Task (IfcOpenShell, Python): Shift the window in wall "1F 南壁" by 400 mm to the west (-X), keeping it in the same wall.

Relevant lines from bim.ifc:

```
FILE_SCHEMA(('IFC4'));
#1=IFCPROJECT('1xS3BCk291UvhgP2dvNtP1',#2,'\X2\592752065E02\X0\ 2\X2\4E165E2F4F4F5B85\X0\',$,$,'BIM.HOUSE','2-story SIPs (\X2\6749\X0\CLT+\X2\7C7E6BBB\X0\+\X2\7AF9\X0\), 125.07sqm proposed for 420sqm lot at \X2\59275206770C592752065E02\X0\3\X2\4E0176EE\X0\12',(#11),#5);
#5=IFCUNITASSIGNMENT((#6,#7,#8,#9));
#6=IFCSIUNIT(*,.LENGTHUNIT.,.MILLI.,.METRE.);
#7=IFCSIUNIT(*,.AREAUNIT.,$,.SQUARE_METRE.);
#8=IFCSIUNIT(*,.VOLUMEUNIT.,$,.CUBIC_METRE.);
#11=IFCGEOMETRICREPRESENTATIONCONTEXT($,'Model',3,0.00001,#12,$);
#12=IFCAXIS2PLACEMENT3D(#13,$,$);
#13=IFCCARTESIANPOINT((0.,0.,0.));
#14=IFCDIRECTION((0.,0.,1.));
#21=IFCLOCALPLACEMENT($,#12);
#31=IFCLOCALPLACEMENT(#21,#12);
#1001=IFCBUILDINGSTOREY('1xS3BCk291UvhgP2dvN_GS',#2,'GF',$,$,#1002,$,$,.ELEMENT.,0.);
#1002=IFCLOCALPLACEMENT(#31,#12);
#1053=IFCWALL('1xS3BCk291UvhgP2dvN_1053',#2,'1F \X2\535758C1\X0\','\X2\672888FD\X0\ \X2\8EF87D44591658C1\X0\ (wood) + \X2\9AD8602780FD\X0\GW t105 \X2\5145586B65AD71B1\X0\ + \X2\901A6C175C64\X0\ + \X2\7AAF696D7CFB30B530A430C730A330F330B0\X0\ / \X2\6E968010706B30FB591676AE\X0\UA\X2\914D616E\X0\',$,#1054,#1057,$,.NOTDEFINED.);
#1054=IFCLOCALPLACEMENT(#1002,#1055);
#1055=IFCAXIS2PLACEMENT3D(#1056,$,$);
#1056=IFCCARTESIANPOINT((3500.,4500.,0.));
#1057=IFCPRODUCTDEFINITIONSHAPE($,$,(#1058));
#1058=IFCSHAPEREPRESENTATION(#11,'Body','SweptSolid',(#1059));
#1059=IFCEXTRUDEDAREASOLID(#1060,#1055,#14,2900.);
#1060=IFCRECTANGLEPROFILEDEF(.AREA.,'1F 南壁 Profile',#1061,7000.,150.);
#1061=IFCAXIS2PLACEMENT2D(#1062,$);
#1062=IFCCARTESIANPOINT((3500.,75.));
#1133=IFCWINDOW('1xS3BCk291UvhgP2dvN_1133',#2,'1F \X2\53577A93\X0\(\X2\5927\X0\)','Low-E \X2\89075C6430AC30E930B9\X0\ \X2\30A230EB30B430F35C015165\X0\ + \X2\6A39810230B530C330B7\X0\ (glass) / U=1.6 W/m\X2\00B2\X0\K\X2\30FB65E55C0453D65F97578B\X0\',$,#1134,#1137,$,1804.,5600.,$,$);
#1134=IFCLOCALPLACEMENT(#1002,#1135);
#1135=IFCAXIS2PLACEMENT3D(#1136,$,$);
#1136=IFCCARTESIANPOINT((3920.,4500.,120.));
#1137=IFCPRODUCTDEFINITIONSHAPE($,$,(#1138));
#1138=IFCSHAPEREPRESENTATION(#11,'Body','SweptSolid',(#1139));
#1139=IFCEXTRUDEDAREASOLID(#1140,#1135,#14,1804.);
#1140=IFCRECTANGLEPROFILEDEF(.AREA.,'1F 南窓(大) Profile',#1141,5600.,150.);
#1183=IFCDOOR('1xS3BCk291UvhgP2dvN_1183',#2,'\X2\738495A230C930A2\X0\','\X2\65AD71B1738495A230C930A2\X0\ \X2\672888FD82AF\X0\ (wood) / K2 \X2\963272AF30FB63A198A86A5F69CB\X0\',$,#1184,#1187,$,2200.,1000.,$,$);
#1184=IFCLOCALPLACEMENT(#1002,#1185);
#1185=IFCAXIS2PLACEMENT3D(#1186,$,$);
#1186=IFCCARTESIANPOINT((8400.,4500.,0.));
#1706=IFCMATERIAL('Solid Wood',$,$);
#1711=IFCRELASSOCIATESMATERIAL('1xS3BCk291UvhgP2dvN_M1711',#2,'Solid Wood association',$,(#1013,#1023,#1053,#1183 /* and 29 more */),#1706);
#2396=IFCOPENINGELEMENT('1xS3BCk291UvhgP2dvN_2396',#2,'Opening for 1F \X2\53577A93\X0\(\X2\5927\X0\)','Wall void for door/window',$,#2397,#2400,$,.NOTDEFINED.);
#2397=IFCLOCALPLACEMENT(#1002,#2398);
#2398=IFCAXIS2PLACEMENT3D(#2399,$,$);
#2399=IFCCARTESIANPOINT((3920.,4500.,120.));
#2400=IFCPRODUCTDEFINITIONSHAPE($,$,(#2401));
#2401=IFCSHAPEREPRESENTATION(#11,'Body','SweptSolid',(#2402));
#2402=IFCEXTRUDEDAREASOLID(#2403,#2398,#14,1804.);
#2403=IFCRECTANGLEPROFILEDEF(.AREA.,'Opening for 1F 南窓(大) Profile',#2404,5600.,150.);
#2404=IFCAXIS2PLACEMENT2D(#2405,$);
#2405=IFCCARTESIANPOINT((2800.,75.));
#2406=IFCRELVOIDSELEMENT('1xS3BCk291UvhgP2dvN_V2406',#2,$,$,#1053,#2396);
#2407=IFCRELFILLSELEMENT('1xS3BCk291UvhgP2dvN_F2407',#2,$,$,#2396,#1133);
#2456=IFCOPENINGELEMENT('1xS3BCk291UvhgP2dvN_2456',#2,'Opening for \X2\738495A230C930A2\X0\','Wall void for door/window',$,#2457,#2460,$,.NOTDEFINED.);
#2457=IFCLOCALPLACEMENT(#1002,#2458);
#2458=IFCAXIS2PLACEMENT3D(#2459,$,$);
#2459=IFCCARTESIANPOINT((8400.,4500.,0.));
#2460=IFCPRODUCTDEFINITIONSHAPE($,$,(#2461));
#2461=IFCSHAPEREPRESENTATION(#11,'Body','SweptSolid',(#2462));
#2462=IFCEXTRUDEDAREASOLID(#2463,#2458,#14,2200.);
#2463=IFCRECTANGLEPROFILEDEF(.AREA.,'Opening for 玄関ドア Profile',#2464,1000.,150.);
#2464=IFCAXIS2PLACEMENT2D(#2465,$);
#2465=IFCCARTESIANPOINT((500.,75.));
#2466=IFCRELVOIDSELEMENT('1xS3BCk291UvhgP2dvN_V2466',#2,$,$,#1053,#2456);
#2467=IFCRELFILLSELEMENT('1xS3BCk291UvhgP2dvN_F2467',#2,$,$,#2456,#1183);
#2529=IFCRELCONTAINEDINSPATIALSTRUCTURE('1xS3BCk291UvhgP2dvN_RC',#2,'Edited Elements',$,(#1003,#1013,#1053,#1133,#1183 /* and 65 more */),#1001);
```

```python
import ifcopenshell
import ifcopenshell.api.geometry
import ifcopenshell.util.placement
import ifcopenshell.util.unit

model = ifcopenshell.open("bim.ifc")
unit_scale = ifcopenshell.util.unit.calculate_unit_scale(model)

window = model.by_id(1133)
opening = window.FillsVoids[0].RelatingOpeningElement
wall = opening.VoidsElements[0].RelatingBuildingElement

wall_matrix = ifcopenshell.util.placement.get_local_placement(wall.ObjectPlacement)
shift = wall_matrix[:3, 0] * -0.4 / unit_scale
before = ifcopenshell.util.placement.get_local_placement(window.ObjectPlacement)[:3, 3].copy()

# The window is not placed relative to its opening, so move both.
for product in (opening, window):
    matrix = ifcopenshell.util.placement.get_local_placement(product.ObjectPlacement)
    matrix[:3, 3] += shift
    ifcopenshell.api.geometry.edit_object_placement(model, product=product, matrix=matrix, is_si=False)

after = ifcopenshell.util.placement.get_local_placement(window.ObjectPlacement)[:3, 3]
print("window moved by", (after - before).round(3) + 0.0)

model.write("bim-out.ifc")
```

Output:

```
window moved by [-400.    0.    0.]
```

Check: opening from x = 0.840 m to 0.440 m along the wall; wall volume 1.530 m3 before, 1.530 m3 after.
